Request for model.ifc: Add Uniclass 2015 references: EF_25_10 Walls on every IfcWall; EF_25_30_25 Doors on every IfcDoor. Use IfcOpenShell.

First a look at what the model holds.

```python
import ifcopenshell

model = ifcopenshell.open("model.ifc")
print(model.schema)
print("classifications:", [c.Name for c in model.by_type("IfcClassification")])
for ifc_class in ("IfcDoor", "IfcRoof", "IfcStair", "IfcWall", "IfcWindow"):
    print(ifc_class, len(model.by_type(ifc_class)))
```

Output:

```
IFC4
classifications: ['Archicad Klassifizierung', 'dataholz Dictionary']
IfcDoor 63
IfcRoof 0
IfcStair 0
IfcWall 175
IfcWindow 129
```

```python
import ifcopenshell
import ifcopenshell.api.classification

model = ifcopenshell.open("model.ifc")

system = ifcopenshell.api.classification.add_classification(model, classification="Uniclass 2015")

codes = {
    "IfcWall": ("EF_25_10", "Walls"),
    "IfcDoor": ("EF_25_30_25", "Doors"),
}
for ifc_class, (code, name) in codes.items():
    products = model.by_type(ifc_class)
    ifcopenshell.api.classification.add_reference(
        model, products=products, classification=system, identification=code, name=name
    )
    print(code, len(products))

model.write("model_rev.ifc")
```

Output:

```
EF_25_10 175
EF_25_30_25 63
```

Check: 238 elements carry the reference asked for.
